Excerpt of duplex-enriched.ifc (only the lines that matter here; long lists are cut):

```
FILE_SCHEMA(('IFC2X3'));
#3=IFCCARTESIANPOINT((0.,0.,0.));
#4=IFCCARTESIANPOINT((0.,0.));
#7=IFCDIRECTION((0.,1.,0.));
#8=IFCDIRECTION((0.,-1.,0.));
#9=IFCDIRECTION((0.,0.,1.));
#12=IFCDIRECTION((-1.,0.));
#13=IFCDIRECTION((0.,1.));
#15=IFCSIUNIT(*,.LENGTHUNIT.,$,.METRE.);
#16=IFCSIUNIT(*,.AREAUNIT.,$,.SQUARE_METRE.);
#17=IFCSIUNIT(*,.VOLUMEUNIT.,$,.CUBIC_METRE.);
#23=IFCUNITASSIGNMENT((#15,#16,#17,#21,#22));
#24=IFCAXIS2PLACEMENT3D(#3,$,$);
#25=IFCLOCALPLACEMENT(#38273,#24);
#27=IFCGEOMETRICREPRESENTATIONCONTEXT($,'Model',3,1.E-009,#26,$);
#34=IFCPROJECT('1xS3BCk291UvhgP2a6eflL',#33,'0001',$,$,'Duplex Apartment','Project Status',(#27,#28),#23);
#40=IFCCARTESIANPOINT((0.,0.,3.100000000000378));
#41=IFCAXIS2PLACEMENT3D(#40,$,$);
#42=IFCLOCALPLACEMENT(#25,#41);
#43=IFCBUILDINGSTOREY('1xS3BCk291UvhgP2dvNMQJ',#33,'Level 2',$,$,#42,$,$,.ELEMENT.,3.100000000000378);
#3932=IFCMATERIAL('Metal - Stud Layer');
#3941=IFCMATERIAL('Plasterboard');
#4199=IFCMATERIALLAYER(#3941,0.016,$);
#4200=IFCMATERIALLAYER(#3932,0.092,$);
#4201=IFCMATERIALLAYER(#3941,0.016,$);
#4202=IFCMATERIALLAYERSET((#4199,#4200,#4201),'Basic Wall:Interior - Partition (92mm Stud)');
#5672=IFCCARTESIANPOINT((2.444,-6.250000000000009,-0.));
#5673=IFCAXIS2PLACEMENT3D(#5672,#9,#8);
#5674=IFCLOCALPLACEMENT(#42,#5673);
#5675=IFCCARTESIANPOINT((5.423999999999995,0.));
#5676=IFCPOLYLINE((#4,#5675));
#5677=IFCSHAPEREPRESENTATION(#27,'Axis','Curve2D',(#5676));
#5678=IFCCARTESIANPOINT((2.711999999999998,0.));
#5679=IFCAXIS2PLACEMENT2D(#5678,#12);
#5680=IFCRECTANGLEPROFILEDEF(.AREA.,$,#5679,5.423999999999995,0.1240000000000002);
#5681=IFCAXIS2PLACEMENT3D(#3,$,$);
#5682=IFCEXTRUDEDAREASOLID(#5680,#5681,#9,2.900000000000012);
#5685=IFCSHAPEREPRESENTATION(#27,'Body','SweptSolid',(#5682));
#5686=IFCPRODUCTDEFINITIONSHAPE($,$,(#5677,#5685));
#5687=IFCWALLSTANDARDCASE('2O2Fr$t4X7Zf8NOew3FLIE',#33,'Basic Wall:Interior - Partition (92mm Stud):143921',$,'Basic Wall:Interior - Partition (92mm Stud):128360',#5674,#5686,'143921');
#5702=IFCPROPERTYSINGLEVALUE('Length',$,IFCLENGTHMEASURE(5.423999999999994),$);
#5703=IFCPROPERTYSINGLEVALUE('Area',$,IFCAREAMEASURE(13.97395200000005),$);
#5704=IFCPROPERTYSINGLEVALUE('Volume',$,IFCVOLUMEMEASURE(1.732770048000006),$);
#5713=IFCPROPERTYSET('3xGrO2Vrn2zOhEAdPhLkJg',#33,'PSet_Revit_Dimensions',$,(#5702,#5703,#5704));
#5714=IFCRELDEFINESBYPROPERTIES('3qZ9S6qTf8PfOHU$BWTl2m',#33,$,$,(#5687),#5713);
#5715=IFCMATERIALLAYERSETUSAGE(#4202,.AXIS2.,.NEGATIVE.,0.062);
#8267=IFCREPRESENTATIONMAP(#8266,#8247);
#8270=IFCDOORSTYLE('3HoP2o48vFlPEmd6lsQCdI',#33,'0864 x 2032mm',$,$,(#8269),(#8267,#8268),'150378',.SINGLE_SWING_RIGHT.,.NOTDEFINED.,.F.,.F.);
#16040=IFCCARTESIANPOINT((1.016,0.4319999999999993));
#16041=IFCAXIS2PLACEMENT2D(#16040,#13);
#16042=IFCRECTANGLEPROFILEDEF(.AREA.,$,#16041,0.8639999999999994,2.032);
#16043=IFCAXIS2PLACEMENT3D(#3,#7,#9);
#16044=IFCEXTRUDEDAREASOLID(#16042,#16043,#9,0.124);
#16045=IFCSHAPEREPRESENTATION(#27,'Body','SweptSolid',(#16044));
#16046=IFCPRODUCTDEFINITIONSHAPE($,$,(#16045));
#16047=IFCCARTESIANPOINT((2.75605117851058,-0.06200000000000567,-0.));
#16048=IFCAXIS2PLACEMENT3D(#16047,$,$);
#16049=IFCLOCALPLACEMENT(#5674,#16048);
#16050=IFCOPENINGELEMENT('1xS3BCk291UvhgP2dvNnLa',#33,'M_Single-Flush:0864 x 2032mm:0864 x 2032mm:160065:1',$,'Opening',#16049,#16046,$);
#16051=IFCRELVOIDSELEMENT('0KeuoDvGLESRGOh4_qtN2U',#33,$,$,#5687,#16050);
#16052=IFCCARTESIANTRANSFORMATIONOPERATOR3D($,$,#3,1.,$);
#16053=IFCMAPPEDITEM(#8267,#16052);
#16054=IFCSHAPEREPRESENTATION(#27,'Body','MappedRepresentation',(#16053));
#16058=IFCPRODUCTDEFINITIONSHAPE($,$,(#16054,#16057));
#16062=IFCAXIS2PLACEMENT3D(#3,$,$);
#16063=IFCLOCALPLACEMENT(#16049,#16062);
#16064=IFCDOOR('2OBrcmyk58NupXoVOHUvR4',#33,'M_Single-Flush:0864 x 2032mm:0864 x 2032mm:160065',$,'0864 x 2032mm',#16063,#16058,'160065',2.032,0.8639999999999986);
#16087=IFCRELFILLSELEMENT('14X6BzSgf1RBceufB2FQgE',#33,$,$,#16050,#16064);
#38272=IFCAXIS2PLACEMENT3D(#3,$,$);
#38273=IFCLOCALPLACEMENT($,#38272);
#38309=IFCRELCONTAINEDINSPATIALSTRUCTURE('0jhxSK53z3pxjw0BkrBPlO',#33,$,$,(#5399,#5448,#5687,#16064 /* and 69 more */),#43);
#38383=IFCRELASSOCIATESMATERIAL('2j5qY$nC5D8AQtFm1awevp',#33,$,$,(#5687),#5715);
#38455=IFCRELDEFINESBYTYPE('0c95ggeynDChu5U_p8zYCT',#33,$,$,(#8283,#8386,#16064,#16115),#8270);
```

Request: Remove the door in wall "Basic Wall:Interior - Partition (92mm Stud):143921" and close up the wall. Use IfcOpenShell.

```python
import ifcopenshell
import ifcopenshell.api.feature
import ifcopenshell.api.pset
import ifcopenshell.api.root
import ifcopenshell.geom
import ifcopenshell.util.element
import ifcopenshell.util.shape
import ifcopenshell.util.unit

model = ifcopenshell.open("duplex-enriched.ifc")
area_scale = ifcopenshell.util.unit.calculate_unit_scale(model, "AREAUNIT")
volume_scale = ifcopenshell.util.unit.calculate_unit_scale(model, "VOLUMEUNIT")
settings = ifcopenshell.geom.settings()


def volume(element):
    """Net volume in cubic metres, openings subtracted."""
    shape = ifcopenshell.geom.create_shape(settings, element)
    return ifcopenshell.util.shape.get_volume(shape.geometry)


door = model.by_guid("2OBrcmyk58NupXoVOHUvR4")
opening = door.FillsVoids[0].RelatingOpeningElement
wall = opening.VoidsElements[0].RelatingBuildingElement
before = volume(wall)

ifcopenshell.api.root.remove_product(model, product=door)
ifcopenshell.api.feature.remove_feature(model, feature=opening)

after = volume(wall)
thickness = 0.124  # wall thickness in metres

# Update the wall's stored quantities.
pset = model.by_id(ifcopenshell.util.element.get_pset(wall, "PSet_Revit_Dimensions", should_inherit=False)["id"])
ifcopenshell.api.pset.edit_pset(model, pset=pset, properties={
    "Area": model.create_entity("IfcAreaMeasure", after / thickness / area_scale),
    "Volume": model.create_entity("IfcVolumeMeasure", after / volume_scale),
})

print(f"wall volume {before:.3f} -> {after:.3f} m3")

model.write("duplex-enriched-out.ifc")
```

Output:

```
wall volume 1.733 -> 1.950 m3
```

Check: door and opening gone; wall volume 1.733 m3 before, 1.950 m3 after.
